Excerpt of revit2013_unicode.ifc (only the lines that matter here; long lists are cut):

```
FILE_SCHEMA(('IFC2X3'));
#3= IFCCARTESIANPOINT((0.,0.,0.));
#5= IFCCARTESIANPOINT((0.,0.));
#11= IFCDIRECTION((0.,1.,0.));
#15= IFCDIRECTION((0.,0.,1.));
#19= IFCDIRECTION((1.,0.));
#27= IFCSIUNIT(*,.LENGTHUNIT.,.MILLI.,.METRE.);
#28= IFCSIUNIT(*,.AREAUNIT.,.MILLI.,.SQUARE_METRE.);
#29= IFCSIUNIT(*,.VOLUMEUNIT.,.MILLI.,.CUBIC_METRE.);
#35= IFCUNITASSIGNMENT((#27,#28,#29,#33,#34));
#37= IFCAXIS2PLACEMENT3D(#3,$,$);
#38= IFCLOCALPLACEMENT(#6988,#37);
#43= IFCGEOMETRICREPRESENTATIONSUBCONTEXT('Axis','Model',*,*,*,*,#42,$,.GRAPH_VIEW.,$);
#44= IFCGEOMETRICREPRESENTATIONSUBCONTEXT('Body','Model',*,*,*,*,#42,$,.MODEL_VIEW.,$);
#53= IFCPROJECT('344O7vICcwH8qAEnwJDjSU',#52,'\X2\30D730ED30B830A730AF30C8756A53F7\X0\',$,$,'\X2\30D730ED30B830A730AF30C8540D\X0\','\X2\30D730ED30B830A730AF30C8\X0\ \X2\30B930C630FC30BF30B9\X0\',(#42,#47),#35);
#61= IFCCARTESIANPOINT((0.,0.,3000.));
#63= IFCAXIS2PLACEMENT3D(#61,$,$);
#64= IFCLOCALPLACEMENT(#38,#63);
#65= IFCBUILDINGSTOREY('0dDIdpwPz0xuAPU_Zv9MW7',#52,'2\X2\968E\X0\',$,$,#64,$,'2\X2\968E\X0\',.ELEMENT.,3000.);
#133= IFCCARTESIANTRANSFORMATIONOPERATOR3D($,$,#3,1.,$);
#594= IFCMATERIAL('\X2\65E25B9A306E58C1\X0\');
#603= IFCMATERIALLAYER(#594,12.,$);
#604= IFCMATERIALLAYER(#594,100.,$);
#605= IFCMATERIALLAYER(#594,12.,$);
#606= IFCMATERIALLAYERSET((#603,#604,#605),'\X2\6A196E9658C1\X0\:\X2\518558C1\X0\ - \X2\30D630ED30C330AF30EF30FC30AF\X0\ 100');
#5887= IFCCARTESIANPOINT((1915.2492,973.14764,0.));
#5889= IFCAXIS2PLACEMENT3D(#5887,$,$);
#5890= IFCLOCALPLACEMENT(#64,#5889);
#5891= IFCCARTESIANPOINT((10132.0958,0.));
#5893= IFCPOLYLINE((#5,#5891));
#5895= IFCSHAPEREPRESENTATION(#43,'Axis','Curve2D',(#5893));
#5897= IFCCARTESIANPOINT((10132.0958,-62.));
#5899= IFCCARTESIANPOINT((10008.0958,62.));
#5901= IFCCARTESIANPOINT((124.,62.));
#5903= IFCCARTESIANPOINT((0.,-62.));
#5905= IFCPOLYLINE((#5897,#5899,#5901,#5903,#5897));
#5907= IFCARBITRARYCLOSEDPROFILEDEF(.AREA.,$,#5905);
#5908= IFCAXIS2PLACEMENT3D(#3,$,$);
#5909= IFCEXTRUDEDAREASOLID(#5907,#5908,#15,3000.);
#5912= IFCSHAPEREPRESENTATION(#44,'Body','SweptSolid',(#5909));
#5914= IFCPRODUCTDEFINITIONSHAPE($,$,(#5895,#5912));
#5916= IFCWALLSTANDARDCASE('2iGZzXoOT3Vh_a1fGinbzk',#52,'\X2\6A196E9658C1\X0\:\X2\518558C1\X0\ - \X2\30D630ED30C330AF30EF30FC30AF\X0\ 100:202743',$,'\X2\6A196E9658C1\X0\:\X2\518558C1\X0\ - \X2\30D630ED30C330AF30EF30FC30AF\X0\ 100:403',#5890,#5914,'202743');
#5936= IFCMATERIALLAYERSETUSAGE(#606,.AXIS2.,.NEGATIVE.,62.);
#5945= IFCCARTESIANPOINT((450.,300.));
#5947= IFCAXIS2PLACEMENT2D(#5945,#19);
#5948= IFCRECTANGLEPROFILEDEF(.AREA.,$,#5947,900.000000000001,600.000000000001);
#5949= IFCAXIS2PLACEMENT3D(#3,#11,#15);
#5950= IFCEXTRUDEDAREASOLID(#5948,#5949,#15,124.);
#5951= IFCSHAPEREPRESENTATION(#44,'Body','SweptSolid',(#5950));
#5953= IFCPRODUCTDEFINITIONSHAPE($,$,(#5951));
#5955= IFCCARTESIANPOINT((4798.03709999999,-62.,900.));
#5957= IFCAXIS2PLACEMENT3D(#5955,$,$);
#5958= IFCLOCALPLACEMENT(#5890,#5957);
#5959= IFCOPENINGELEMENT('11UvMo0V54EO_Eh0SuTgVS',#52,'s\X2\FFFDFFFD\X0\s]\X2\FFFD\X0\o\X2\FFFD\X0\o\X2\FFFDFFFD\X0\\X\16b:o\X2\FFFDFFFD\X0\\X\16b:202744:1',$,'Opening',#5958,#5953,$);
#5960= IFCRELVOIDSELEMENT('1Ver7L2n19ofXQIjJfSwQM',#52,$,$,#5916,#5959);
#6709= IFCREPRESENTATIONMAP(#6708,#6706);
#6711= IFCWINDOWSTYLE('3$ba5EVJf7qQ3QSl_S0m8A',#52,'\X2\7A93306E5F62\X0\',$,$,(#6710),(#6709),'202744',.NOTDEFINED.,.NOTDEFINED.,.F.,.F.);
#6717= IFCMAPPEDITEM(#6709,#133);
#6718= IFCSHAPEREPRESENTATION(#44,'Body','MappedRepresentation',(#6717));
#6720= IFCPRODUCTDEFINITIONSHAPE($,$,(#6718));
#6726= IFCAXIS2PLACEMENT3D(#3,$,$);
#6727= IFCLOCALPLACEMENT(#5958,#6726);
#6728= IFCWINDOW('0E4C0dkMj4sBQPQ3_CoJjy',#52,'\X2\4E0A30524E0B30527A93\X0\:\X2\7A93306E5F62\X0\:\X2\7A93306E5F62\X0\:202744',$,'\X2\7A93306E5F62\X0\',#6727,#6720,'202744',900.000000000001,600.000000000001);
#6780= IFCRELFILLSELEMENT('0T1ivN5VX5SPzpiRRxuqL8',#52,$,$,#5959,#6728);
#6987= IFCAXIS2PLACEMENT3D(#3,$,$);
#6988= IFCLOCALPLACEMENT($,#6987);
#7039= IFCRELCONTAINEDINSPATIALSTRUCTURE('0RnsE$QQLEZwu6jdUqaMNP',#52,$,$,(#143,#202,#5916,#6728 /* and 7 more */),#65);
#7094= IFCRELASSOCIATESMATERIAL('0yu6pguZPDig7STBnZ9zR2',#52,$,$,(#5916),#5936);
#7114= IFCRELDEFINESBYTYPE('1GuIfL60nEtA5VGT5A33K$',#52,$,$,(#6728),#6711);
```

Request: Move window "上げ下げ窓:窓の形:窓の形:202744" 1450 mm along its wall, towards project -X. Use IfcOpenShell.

```python
import ifcopenshell
import ifcopenshell.api.geometry
import ifcopenshell.util.placement
import ifcopenshell.util.unit

model = ifcopenshell.open("revit2013_unicode.ifc")
unit_scale = ifcopenshell.util.unit.calculate_unit_scale(model)

window = model.by_guid("0E4C0dkMj4sBQPQ3_CoJjy")
opening = window.FillsVoids[0].RelatingOpeningElement
wall = opening.VoidsElements[0].RelatingBuildingElement

wall_matrix = ifcopenshell.util.placement.get_local_placement(wall.ObjectPlacement)
shift = wall_matrix[:3, 0] * -1.45 / unit_scale
before = ifcopenshell.util.placement.get_local_placement(window.ObjectPlacement)[:3, 3].copy()

# The window is placed relative to its opening, so it follows when the opening moves.
matrix = ifcopenshell.util.placement.get_local_placement(opening.ObjectPlacement)
matrix[:3, 3] += shift
ifcopenshell.api.geometry.edit_object_placement(
    model, product=opening, matrix=matrix, is_si=False, should_transform_children=True
)

after = ifcopenshell.util.placement.get_local_placement(window.ObjectPlacement)[:3, 3]
print("window moved by", (after - before).round(3) + 0.0)

model.write("revit2013_unicode_v2.ifc")
```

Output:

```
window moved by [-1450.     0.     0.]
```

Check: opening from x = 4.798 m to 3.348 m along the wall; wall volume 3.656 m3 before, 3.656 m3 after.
